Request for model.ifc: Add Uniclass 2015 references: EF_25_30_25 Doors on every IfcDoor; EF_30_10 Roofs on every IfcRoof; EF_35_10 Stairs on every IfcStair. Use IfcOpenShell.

First a look at what the model holds.

```python
import ifcopenshell

model = ifcopenshell.open("model.ifc")
print(model.schema)
print("classifications:", [c.Name for c in model.by_type("IfcClassification")])
for ifc_class in ("IfcDoor", "IfcRoof", "IfcStair", "IfcWall", "IfcWindow"):
    print(ifc_class, len(model.by_type(ifc_class)))
```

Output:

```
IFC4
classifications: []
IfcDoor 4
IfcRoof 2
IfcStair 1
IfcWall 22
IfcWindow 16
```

```python
import ifcopenshell
import ifcopenshell.api.classification

model = ifcopenshell.open("model.ifc")

system = ifcopenshell.api.classification.add_classification(model, classification="Uniclass 2015")

codes = {
    "IfcDoor": ("EF_25_30_25", "Doors"),
    "IfcRoof": ("EF_30_10", "Roofs"),
    "IfcStair": ("EF_35_10", "Stairs"),
}
for ifc_class, (code, name) in codes.items():
    products = model.by_type(ifc_class)
    ifcopenshell.api.classification.add_reference(
        model, products=products, classification=system, identification=code, name=name
    )
    print(code, len(products))

model.write("model_updated.ifc")
```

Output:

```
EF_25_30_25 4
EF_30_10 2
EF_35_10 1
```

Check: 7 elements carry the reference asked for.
